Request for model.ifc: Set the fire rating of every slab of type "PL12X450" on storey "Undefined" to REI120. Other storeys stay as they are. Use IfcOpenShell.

First a look at what the model holds.

```python
import ifcopenshell
import ifcopenshell.util.element

model = ifcopenshell.open("model.ifc")
print(model.schema)
storey = next(s for s in model.by_type("IfcBuildingStorey") if s.Name == "Undefined")
slabs = [e for e in ifcopenshell.util.element.get_decomposition(storey) if e.is_a("IfcSlab")]
seen = {}
for e in slabs:
    element_type = ifcopenshell.util.element.get_type(e)
    key = (element_type.Name if element_type != e and element_type else None, ifcopenshell.util.element.get_pset(e, "Pset_SlabCommon", "FireRating"))
    seen[key] = seen.get(key, 0) + 1
for (name, value), count in sorted(seen.items(), key=str):
    print(count, "x", name, "|", value)
```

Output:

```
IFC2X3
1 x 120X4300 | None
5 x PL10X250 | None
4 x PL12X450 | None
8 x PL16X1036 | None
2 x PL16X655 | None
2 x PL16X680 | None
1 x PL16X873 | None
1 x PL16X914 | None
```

```python
import ifcopenshell
import ifcopenshell.api.pset
import ifcopenshell.util.element

model = ifcopenshell.open("model.ifc")

storey = next(s for s in model.by_type("IfcBuildingStorey") if s.Name == "Undefined")
slabs = [e for e in ifcopenshell.util.element.get_decomposition(storey) if e.is_a("IfcSlab")]

count = 0
for e in slabs:
    element_type = ifcopenshell.util.element.get_type(e)
    if element_type in (None, e) or element_type.Name != "PL12X450":
        continue
    # add_pset returns the element's existing set when there is one.
    pset = ifcopenshell.api.pset.add_pset(model, product=e, name="Pset_SlabCommon")
    ifcopenshell.api.pset.edit_pset(model, pset=pset, properties={"FireRating": "REI120"})
    count += 1

print(count, "slabs updated")

model.write("model_updated.ifc")
```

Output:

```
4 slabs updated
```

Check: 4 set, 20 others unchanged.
